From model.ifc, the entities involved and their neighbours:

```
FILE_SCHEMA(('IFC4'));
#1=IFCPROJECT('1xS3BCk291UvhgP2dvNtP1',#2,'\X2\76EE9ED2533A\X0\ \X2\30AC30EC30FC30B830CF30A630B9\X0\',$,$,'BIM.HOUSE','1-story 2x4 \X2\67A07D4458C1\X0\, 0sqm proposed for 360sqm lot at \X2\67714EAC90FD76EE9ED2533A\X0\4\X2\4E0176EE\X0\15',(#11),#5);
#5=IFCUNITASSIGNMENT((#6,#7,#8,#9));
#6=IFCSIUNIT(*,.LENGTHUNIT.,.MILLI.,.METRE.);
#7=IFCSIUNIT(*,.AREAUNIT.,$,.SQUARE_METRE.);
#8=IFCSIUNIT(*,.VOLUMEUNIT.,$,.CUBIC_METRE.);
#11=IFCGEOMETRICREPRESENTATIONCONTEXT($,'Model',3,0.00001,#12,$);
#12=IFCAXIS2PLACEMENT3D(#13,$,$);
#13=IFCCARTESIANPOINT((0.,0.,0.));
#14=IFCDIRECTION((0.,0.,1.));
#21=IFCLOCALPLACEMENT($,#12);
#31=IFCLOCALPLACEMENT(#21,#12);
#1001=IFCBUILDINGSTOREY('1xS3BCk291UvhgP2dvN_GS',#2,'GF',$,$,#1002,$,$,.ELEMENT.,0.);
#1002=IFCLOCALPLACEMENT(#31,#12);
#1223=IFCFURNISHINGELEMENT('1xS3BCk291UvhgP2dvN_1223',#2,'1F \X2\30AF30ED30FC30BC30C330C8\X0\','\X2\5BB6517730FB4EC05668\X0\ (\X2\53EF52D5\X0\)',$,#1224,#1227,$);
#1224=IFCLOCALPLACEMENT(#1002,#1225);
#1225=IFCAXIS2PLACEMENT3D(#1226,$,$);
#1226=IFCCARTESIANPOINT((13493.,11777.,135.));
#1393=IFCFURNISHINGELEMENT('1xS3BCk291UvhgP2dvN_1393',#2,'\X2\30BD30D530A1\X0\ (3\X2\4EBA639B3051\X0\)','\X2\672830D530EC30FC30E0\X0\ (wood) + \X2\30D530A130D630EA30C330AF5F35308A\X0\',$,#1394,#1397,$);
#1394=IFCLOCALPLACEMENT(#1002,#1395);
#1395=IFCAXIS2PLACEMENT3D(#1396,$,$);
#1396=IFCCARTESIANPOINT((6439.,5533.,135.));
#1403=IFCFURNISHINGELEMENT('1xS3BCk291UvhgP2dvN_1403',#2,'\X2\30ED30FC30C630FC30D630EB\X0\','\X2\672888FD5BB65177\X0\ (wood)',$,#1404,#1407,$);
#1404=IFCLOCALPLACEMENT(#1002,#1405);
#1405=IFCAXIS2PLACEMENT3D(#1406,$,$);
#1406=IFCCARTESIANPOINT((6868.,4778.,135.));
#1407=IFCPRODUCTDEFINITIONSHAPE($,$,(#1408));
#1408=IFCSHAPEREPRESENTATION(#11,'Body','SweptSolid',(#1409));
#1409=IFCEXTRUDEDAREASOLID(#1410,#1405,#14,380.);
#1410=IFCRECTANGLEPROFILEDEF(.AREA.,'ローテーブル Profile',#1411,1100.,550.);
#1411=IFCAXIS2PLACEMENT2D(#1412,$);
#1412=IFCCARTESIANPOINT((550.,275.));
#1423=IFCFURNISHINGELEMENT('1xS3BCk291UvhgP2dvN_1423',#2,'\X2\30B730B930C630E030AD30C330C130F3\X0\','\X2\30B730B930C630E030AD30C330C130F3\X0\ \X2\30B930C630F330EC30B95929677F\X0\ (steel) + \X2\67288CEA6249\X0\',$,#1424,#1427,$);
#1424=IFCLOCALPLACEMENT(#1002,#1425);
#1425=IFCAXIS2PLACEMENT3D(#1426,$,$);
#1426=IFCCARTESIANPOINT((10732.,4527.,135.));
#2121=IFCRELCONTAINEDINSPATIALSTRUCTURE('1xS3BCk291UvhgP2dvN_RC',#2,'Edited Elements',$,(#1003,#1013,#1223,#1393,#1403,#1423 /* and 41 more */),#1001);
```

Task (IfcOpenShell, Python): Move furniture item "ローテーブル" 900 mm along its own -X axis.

```python
import ifcopenshell
import ifcopenshell.api.geometry
import ifcopenshell.util.placement

model = ifcopenshell.open("model.ifc")

item = model.by_guid("1xS3BCk291UvhgP2dvN_1403")
matrix = ifcopenshell.util.placement.get_local_placement(item.ObjectPlacement)
matrix[:3, 3] -= matrix[:3, 0] * 900.0
ifcopenshell.api.geometry.edit_object_placement(model, product=item, matrix=matrix, is_si=False)

print(ifcopenshell.util.placement.get_local_placement(item.ObjectPlacement).round(3) + 0.0)

model.write("model-out.ifc")
```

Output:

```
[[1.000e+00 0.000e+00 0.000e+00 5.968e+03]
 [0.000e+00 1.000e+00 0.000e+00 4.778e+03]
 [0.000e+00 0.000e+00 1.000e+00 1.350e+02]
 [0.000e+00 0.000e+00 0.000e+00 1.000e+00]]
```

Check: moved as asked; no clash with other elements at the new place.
